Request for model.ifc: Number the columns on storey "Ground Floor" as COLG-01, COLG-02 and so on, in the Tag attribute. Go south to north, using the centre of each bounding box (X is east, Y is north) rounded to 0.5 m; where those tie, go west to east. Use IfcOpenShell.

First a look at what the model holds.

```python
import ifcopenshell
import ifcopenshell.util.element
import ifcopenshell.util.placement

model = ifcopenshell.open("model.ifc")
print(model.schema)
storey = next(s for s in model.by_type("IfcBuildingStorey") if s.Name == "Ground Floor")
columns = [e for e in ifcopenshell.util.element.get_decomposition(storey) if e.is_a("IfcColumn")]
for e in sorted(columns, key=lambda e: e.id()):
    origin = ifcopenshell.util.placement.get_local_placement(e.ObjectPlacement)[:3, 3]
    print(e.id(), e.Tag, e.Name, origin.round(2) + 0.0, sep=" | ")
```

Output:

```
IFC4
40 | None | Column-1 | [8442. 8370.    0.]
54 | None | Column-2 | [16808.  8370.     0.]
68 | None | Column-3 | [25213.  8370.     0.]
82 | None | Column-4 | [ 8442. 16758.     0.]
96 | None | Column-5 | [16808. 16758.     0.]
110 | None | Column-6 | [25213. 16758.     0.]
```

```python
import ifcopenshell
import ifcopenshell.geom
import ifcopenshell.util.element
import ifcopenshell.util.shape

model = ifcopenshell.open("model.ifc")
settings = ifcopenshell.geom.settings()
settings.set("use-world-coords", True)


def centre(element):
    shape = ifcopenshell.geom.create_shape(settings, element)
    return ifcopenshell.util.shape.get_bbox_centroid(shape.geometry)


storey = next(s for s in model.by_type("IfcBuildingStorey") if s.Name == "Ground Floor")
columns = [e for e in ifcopenshell.util.element.get_decomposition(storey) if e.is_a("IfcColumn")]

# Insertion points can sit at a corner or the storey origin, so sort by the geometry (in metres).
centres = {e: centre(e) for e in columns}
columns.sort(key=lambda e: (round(centres[e][1] / 0.5), centres[e][0]))

for i, e in enumerate(columns, start=1):
    number = f"COLG-{i:02d}"
    e.Tag = number
    print(e.id(), number)

model.write("model_rev.ifc")
```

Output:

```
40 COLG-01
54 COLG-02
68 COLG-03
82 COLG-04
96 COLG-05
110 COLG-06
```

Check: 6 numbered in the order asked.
